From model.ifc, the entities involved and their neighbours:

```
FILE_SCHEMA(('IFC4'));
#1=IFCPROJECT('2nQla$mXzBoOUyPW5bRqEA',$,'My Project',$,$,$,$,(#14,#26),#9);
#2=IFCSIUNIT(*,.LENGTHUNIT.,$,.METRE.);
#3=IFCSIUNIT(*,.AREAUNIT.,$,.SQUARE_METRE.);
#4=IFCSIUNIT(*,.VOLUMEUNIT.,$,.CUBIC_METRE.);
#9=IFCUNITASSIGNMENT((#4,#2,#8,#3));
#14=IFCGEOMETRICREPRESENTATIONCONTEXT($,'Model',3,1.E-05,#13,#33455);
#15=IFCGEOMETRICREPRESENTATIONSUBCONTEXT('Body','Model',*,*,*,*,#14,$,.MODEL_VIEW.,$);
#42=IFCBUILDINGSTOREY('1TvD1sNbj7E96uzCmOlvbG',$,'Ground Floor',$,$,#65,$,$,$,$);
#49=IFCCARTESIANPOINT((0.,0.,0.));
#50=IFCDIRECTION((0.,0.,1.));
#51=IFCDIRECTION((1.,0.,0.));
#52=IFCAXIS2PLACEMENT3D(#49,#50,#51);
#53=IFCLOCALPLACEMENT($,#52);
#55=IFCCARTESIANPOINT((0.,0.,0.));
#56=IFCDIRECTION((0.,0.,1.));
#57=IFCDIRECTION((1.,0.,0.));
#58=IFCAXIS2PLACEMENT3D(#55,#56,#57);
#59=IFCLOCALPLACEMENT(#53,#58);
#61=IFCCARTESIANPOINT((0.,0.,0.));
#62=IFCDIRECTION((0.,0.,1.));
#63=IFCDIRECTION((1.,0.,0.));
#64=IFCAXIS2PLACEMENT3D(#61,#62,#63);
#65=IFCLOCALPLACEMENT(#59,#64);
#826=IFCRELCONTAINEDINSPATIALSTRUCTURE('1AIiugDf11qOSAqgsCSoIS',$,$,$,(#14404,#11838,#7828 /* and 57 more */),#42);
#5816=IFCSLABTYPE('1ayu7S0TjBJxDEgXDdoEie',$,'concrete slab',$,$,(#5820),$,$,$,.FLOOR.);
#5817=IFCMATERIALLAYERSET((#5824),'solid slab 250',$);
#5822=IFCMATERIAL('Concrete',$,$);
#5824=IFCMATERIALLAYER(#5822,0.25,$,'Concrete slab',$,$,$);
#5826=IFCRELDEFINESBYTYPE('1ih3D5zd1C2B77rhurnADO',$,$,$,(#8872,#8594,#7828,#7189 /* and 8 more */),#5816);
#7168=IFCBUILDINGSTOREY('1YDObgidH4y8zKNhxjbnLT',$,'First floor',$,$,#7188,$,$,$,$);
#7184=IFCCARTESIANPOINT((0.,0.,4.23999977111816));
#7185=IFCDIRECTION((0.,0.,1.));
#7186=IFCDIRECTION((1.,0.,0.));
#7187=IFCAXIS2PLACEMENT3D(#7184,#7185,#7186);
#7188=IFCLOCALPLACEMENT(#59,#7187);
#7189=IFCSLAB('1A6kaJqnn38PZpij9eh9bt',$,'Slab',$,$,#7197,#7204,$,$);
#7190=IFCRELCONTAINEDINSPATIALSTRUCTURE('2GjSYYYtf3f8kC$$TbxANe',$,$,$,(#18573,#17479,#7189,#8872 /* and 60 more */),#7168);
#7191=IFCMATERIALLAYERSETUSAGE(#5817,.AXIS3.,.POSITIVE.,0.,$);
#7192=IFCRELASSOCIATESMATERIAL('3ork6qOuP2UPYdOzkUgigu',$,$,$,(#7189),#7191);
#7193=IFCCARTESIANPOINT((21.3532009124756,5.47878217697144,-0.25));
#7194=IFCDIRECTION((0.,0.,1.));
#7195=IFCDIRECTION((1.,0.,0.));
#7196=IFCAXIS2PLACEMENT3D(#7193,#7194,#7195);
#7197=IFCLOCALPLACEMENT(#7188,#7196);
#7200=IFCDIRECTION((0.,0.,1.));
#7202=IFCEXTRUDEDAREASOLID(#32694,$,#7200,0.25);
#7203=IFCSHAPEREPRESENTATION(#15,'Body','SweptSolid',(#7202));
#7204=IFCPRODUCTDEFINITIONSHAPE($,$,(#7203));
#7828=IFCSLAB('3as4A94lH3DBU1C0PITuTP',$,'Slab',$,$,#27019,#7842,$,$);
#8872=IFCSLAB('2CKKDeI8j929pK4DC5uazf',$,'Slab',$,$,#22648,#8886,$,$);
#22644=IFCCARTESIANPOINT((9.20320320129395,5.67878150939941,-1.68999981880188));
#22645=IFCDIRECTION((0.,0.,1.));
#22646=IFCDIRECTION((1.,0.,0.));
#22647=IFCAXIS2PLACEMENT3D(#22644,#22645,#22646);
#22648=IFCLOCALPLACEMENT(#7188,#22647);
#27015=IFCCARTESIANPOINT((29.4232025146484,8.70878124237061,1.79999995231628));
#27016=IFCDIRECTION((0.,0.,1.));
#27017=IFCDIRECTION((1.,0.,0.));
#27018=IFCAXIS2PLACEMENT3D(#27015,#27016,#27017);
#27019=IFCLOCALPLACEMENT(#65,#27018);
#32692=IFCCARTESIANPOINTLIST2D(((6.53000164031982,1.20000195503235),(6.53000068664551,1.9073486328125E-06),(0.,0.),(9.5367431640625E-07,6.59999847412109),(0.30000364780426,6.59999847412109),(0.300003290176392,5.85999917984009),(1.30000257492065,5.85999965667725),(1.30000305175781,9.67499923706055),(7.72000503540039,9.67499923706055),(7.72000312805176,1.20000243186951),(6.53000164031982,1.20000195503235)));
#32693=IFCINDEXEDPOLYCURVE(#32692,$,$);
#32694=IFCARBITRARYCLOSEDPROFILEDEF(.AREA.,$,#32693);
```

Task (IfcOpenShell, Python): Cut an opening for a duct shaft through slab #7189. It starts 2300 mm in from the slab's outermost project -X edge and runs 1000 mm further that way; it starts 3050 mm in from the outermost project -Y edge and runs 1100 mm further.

```python
import numpy as np
import ifcopenshell
import ifcopenshell.api.feature
import ifcopenshell.api.geometry
import ifcopenshell.api.root
import ifcopenshell.geom
import ifcopenshell.util.placement
import ifcopenshell.util.representation
import ifcopenshell.util.shape
import ifcopenshell.util.unit

model = ifcopenshell.open("model.ifc")
unit_scale = ifcopenshell.util.unit.calculate_unit_scale(model)
settings = ifcopenshell.geom.settings()


def volume(element):
    """Net volume in cubic metres, openings subtracted."""
    shape = ifcopenshell.geom.create_shape(settings, element)
    return ifcopenshell.util.shape.get_volume(shape.geometry)


slab = model.by_guid("1A6kaJqnn38PZpij9eh9bt")
before = volume(slab)

# Extent in the slab's own axes, in metres. The edges named are its -X and -Y sides.
slab_shape = ifcopenshell.geom.create_shape(settings, slab)
vertices = ifcopenshell.util.shape.get_vertices(slab_shape.geometry)
x_min, y_min, bottom = vertices.min(axis=0)
top = vertices[:, 2].max()

opening = ifcopenshell.api.root.create_entity(model, ifc_class="IfcOpeningElement", name="Duct shaft opening", predefined_type="OPENING")
context = ifcopenshell.util.representation.get_context(model, "Model", "Body", "MODEL_VIEW")
width, depth = 1, 1.1
outline = [(0.0, 0.0), (width, 0.0), (width, depth), (0.0, depth), (0.0, 0.0)]
# Overshoot both faces by 50 mm so the cut is clean.
shape = ifcopenshell.api.geometry.add_slab_representation(
    model, context=context, depth=top - bottom + 0.1, polyline=outline
)
ifcopenshell.api.geometry.assign_representation(model, product=opening, representation=shape)

matrix = ifcopenshell.util.placement.get_local_placement(slab.ObjectPlacement)
matrix[:, 3] = matrix @ np.append(np.array([x_min + 2.3, y_min + 3.05, bottom - 0.05]) / unit_scale, 1.0)
ifcopenshell.api.geometry.edit_object_placement(model, product=opening, matrix=matrix, is_si=False)
ifcopenshell.api.feature.add_feature(model, feature=opening, element=slab)

after = volume(slab)

print(f"slab volume {before:.3f} -> {after:.3f} m3")

model.write("model_updated.ifc")
```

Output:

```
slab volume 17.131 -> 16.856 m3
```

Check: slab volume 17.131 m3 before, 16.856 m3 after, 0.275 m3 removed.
